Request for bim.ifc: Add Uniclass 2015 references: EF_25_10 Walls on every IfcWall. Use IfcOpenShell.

First a look at what the model holds.

```python
import ifcopenshell

model = ifcopenshell.open("bim.ifc")
print(model.schema)
print("classifications:", [c.Name for c in model.by_type("IfcClassification")])
for ifc_class in ("IfcDoor", "IfcRoof", "IfcStair", "IfcWall", "IfcWindow"):
    print(ifc_class, len(model.by_type(ifc_class)))
```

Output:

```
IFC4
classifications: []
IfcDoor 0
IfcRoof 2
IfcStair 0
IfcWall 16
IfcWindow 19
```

```python
import ifcopenshell
import ifcopenshell.api.classification

model = ifcopenshell.open("bim.ifc")

system = ifcopenshell.api.classification.add_classification(model, classification="Uniclass 2015")

codes = {
    "IfcWall": ("EF_25_10", "Walls"),
}
for ifc_class, (code, name) in codes.items():
    products = model.by_type(ifc_class)
    ifcopenshell.api.classification.add_reference(
        model, products=products, classification=system, identification=code, name=name
    )
    print(code, len(products))

model.write("bim_updated.ifc")
```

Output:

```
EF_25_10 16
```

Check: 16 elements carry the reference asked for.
